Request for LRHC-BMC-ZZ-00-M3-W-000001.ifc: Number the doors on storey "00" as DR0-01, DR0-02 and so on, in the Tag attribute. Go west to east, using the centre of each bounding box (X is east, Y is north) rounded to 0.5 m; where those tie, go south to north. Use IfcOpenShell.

First a look at what the model holds.

```python
import ifcopenshell
import ifcopenshell.util.element
import ifcopenshell.util.placement

model = ifcopenshell.open("LRHC-BMC-ZZ-00-M3-W-000001.ifc")
print(model.schema)
storey = next(s for s in model.by_type("IfcBuildingStorey") if s.Name == "00")
doors = [e for e in ifcopenshell.util.element.get_decomposition(storey) if e.is_a("IfcDoor")]
for e in sorted(doors, key=lambda e: e.id()):
    origin = ifcopenshell.util.placement.get_local_placement(e.ObjectPlacement)[:3, 3]
    print(e.id(), e.Tag, e.Name, origin.round(2) + 0.0, sep=" | ")
```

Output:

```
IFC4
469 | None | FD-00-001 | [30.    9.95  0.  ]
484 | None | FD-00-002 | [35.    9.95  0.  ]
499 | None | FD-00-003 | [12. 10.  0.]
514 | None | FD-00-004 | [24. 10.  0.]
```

```python
import ifcopenshell
import ifcopenshell.geom
import ifcopenshell.util.element
import ifcopenshell.util.shape

model = ifcopenshell.open("LRHC-BMC-ZZ-00-M3-W-000001.ifc")
settings = ifcopenshell.geom.settings()
settings.set("use-world-coords", True)


def centre(element):
    shape = ifcopenshell.geom.create_shape(settings, element)
    return ifcopenshell.util.shape.get_bbox_centroid(shape.geometry)


storey = next(s for s in model.by_type("IfcBuildingStorey") if s.Name == "00")
doors = [e for e in ifcopenshell.util.element.get_decomposition(storey) if e.is_a("IfcDoor")]

# Insertion points can sit at a corner or the storey origin, so sort by the geometry (in metres).
centres = {e: centre(e) for e in doors}
doors.sort(key=lambda e: (round(centres[e][0] / 0.5), centres[e][1]))

for i, e in enumerate(doors, start=1):
    number = f"DR0-{i:02d}"
    e.Tag = number
    print(e.id(), number)

model.write("LRHC-BMC-ZZ-00-M3-W-000001_updated.ifc")
```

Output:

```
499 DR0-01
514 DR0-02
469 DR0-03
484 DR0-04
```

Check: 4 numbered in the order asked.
